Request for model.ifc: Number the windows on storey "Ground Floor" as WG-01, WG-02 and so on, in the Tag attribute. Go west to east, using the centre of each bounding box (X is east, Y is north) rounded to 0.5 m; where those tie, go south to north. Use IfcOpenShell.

First a look at what the model holds.

```python
import ifcopenshell
import ifcopenshell.util.element
import ifcopenshell.util.placement

model = ifcopenshell.open("model.ifc")
print(model.schema)
storey = next(s for s in model.by_type("IfcBuildingStorey") if s.Name == "Ground Floor")
windows = [e for e in ifcopenshell.util.element.get_decomposition(storey) if e.is_a("IfcWindow")]
for e in sorted(windows, key=lambda e: e.id()):
    origin = ifcopenshell.util.placement.get_local_placement(e.ObjectPlacement)[:3, 3]
    print(e.id(), e.Tag, e.Name, origin.round(2) + 0.0, sep=" | ")
```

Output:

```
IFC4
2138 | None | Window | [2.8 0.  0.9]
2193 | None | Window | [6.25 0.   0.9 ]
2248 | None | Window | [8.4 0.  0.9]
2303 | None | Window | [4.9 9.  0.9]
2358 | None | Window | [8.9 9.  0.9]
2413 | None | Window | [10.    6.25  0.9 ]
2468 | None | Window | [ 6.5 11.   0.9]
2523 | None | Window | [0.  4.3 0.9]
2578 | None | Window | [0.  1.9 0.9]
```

```python
import ifcopenshell
import ifcopenshell.geom
import ifcopenshell.util.element
import ifcopenshell.util.shape

model = ifcopenshell.open("model.ifc")
settings = ifcopenshell.geom.settings()
settings.set("use-world-coords", True)


def centre(element):
    shape = ifcopenshell.geom.create_shape(settings, element)
    return ifcopenshell.util.shape.get_bbox_centroid(shape.geometry)


storey = next(s for s in model.by_type("IfcBuildingStorey") if s.Name == "Ground Floor")
windows = [e for e in ifcopenshell.util.element.get_decomposition(storey) if e.is_a("IfcWindow")]

# Insertion points can sit at a corner or the storey origin, so sort by the geometry (in metres).
centres = {e: centre(e) for e in windows}
windows.sort(key=lambda e: (round(centres[e][0] / 0.5), centres[e][1]))

for i, e in enumerate(windows, start=1):
    number = f"WG-{i:02d}"
    e.Tag = number
    print(e.id(), number)

model.write("model_edited.ifc")
```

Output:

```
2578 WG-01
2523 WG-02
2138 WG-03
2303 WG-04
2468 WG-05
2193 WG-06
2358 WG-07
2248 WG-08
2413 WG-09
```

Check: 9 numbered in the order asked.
